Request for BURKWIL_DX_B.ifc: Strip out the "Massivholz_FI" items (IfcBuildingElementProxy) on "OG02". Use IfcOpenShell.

First a look at what the model holds.

```python
import ifcopenshell
import ifcopenshell.util.element

model = ifcopenshell.open("BURKWIL_DX_B.ifc")
print(model.schema)
storey = next(s for s in model.by_type("IfcBuildingStorey") if s.Name == "OG02")
proxies = [e for e in ifcopenshell.util.element.get_decomposition(storey) if e.is_a("IfcBuildingElementProxy")]
seen = {}
for e in proxies:
    element_type = ifcopenshell.util.element.get_type(e)
    name = element_type.Name if element_type not in (None, e) else None
    seen[name] = seen.get(name, 0) + 1
for name, count in sorted(seen.items(), key=str):
    print(count, "x", name)
```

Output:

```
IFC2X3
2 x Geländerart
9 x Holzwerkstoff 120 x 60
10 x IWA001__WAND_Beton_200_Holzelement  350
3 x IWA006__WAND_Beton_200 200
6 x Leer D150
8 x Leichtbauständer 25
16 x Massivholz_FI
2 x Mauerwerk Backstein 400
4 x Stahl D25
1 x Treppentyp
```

```python
import ifcopenshell
import ifcopenshell.api.root
import ifcopenshell.util.element

model = ifcopenshell.open("BURKWIL_DX_B.ifc")

storey = next(s for s in model.by_type("IfcBuildingStorey") if s.Name == "OG02")
proxies = [e for e in ifcopenshell.util.element.get_decomposition(storey) if e.is_a("IfcBuildingElementProxy")]
targets = [e for e in proxies if (t := ifcopenshell.util.element.get_type(e)) not in (None, e) and t.Name == "Massivholz_FI"]

for e in targets:
    ifcopenshell.api.root.remove_product(model, product=e)
print(len(targets), "removed")

model.write("BURKWIL_DX_B_rev.ifc")
```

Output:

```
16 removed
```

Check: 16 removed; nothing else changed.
